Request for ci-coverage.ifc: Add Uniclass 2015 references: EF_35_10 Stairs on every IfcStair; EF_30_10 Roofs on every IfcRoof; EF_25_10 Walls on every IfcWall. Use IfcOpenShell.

First a look at what the model holds.

```python
import ifcopenshell

model = ifcopenshell.open("ci-coverage.ifc")
print(model.schema)
print("classifications:", [c.Name for c in model.by_type("IfcClassification")])
for ifc_class in ("IfcDoor", "IfcRoof", "IfcStair", "IfcWall", "IfcWindow"):
    print(ifc_class, len(model.by_type(ifc_class)))
```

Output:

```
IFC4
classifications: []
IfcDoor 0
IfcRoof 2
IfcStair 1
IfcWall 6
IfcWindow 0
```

```python
import ifcopenshell
import ifcopenshell.api.classification

model = ifcopenshell.open("ci-coverage.ifc")

system = ifcopenshell.api.classification.add_classification(model, classification="Uniclass 2015")

codes = {
    "IfcStair": ("EF_35_10", "Stairs"),
    "IfcRoof": ("EF_30_10", "Roofs"),
    "IfcWall": ("EF_25_10", "Walls"),
}
for ifc_class, (code, name) in codes.items():
    products = model.by_type(ifc_class)
    ifcopenshell.api.classification.add_reference(
        model, products=products, classification=system, identification=code, name=name
    )
    print(code, len(products))

model.write("ci-coverage-out.ifc")
```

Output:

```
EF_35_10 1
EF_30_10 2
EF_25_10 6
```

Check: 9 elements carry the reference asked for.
